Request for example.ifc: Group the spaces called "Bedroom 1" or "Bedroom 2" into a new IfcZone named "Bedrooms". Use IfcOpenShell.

First a look at what the model holds.

```python
import ifcopenshell

model = ifcopenshell.open("example.ifc")
print(model.schema)
seen = {}
for space in model.by_type("IfcSpace"):
    seen[space.LongName] = seen.get(space.LongName, 0) + 1
for name, count in sorted(seen.items(), key=str):
    print(count, "x", name)
print("zones:", [z.Name for z in model.by_type("IfcZone")][:20])
```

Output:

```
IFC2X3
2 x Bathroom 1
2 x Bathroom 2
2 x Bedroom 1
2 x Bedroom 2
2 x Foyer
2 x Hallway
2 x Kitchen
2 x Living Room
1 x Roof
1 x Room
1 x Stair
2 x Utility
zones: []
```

```python
import ifcopenshell
import ifcopenshell.api.group
import ifcopenshell.api.root

model = ifcopenshell.open("example.ifc")

names = {"Bedroom 1", "Bedroom 2"}
spaces = [s for s in model.by_type("IfcSpace") if s.LongName in names]

zone = ifcopenshell.api.root.create_entity(model, ifc_class="IfcZone", name="Bedrooms")
ifcopenshell.api.group.assign_group(model, products=spaces, group=zone)
print(len(spaces), "spaces in", zone.Name)

model.write("example_updated.ifc")
```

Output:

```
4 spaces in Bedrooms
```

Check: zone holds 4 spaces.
